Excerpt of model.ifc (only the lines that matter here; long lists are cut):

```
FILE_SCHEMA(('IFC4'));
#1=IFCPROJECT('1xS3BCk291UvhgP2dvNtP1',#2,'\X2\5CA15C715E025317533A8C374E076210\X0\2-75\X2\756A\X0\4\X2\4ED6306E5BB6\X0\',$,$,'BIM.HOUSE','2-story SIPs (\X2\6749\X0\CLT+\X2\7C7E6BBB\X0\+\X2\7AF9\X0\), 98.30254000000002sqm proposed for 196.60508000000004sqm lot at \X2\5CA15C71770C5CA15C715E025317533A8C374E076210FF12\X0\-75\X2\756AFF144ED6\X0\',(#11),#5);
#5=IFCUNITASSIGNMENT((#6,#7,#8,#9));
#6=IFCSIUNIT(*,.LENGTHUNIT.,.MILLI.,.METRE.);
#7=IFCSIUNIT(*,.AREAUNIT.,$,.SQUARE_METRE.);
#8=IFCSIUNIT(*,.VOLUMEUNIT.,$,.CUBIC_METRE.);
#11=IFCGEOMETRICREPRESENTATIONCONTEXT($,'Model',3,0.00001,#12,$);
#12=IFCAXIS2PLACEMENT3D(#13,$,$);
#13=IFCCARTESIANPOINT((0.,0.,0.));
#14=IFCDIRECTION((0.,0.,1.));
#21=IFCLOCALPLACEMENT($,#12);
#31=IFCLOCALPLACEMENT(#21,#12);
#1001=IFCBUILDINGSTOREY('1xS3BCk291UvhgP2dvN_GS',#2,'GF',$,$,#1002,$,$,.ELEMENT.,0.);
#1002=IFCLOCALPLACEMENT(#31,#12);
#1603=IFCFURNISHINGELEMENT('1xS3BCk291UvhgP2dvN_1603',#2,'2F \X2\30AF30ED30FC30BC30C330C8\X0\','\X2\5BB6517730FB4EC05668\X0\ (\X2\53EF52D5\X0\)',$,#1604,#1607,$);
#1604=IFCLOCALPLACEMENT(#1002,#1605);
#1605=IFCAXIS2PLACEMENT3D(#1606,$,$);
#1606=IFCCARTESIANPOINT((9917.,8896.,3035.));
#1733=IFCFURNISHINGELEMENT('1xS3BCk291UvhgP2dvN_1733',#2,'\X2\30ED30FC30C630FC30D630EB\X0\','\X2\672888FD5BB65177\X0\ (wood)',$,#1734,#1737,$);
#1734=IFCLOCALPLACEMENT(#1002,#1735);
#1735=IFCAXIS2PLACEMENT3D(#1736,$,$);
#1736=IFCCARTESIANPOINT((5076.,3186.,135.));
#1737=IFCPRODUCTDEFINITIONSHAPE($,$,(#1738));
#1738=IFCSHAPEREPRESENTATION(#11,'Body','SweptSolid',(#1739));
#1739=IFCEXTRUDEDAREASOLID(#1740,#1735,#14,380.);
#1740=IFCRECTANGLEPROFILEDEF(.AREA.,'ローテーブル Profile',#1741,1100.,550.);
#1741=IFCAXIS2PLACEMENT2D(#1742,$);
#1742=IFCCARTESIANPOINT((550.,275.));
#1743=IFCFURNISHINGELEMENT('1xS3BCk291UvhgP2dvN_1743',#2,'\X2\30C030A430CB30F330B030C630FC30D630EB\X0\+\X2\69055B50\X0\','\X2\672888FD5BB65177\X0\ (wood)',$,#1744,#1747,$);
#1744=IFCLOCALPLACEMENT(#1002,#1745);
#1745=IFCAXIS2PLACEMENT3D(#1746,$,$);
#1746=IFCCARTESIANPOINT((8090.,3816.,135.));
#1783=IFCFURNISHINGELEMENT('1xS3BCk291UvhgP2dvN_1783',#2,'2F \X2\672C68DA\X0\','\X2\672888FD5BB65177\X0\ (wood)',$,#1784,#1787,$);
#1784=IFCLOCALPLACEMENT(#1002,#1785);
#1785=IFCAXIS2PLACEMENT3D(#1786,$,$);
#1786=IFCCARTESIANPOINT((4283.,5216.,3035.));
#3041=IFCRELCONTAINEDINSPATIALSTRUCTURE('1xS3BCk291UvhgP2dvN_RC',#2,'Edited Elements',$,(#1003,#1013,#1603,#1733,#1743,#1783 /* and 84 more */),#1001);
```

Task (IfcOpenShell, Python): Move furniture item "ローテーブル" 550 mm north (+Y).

```python
import ifcopenshell
import ifcopenshell.api.geometry
import ifcopenshell.util.placement
import ifcopenshell.util.unit

model = ifcopenshell.open("model.ifc")
unit_scale = ifcopenshell.util.unit.calculate_unit_scale(model)

item = model.by_guid("1xS3BCk291UvhgP2dvN_1733")
matrix = ifcopenshell.util.placement.get_local_placement(item.ObjectPlacement)
matrix[1, 3] += 0.55 / unit_scale
ifcopenshell.api.geometry.edit_object_placement(model, product=item, matrix=matrix, is_si=False)

print(ifcopenshell.util.placement.get_local_placement(item.ObjectPlacement).round(3) + 0.0)

model.write("model_updated.ifc")
```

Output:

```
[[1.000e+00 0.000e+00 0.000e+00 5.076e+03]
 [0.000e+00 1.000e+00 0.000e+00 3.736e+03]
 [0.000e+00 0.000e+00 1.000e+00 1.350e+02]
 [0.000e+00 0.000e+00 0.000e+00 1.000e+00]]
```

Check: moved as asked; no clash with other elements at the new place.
